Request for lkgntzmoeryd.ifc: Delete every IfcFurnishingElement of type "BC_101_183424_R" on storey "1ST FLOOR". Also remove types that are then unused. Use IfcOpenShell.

First a look at what the model holds.

```python
import ifcopenshell
import ifcopenshell.util.element

model = ifcopenshell.open("lkgntzmoeryd.ifc")
print(model.schema)
storey = next(s for s in model.by_type("IfcBuildingStorey") if s.Name == "1ST FLOOR")
furniture = [e for e in ifcopenshell.util.element.get_decomposition(storey) if e.is_a("IfcFurnishingElement")]
seen = {}
for e in furniture:
    element_type = ifcopenshell.util.element.get_type(e)
    name = element_type.Name if element_type not in (None, e) else None
    seen[name] = seen.get(name, 0) + 1
for name, count in sorted(seen.items(), key=str):
    print(count, "x", name)
```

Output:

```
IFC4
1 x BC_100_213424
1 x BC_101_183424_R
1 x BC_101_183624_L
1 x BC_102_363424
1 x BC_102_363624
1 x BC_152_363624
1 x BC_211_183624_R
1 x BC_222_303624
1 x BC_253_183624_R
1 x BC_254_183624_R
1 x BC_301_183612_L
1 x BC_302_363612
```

```python
import ifcopenshell
import ifcopenshell.api.root
import ifcopenshell.util.element

model = ifcopenshell.open("lkgntzmoeryd.ifc")

storey = next(s for s in model.by_type("IfcBuildingStorey") if s.Name == "1ST FLOOR")
furniture = [e for e in ifcopenshell.util.element.get_decomposition(storey) if e.is_a("IfcFurnishingElement")]
targets = [e for e in furniture if (t := ifcopenshell.util.element.get_type(e)) not in (None, e) and t.Name == "BC_101_183424_R"]
types = {ifcopenshell.util.element.get_type(e) for e in targets} - {None, *targets}

for e in targets:
    ifcopenshell.api.root.remove_product(model, product=e)
print(len(targets), "removed")

unused = [t for t in types if not ifcopenshell.util.element.get_types(t)]
for t in unused:
    ifcopenshell.api.root.remove_product(model, product=t)
print(len(unused), "unused types removed")

model.write("lkgntzmoeryd_updated.ifc")
```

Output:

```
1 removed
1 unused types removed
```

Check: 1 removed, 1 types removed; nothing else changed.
